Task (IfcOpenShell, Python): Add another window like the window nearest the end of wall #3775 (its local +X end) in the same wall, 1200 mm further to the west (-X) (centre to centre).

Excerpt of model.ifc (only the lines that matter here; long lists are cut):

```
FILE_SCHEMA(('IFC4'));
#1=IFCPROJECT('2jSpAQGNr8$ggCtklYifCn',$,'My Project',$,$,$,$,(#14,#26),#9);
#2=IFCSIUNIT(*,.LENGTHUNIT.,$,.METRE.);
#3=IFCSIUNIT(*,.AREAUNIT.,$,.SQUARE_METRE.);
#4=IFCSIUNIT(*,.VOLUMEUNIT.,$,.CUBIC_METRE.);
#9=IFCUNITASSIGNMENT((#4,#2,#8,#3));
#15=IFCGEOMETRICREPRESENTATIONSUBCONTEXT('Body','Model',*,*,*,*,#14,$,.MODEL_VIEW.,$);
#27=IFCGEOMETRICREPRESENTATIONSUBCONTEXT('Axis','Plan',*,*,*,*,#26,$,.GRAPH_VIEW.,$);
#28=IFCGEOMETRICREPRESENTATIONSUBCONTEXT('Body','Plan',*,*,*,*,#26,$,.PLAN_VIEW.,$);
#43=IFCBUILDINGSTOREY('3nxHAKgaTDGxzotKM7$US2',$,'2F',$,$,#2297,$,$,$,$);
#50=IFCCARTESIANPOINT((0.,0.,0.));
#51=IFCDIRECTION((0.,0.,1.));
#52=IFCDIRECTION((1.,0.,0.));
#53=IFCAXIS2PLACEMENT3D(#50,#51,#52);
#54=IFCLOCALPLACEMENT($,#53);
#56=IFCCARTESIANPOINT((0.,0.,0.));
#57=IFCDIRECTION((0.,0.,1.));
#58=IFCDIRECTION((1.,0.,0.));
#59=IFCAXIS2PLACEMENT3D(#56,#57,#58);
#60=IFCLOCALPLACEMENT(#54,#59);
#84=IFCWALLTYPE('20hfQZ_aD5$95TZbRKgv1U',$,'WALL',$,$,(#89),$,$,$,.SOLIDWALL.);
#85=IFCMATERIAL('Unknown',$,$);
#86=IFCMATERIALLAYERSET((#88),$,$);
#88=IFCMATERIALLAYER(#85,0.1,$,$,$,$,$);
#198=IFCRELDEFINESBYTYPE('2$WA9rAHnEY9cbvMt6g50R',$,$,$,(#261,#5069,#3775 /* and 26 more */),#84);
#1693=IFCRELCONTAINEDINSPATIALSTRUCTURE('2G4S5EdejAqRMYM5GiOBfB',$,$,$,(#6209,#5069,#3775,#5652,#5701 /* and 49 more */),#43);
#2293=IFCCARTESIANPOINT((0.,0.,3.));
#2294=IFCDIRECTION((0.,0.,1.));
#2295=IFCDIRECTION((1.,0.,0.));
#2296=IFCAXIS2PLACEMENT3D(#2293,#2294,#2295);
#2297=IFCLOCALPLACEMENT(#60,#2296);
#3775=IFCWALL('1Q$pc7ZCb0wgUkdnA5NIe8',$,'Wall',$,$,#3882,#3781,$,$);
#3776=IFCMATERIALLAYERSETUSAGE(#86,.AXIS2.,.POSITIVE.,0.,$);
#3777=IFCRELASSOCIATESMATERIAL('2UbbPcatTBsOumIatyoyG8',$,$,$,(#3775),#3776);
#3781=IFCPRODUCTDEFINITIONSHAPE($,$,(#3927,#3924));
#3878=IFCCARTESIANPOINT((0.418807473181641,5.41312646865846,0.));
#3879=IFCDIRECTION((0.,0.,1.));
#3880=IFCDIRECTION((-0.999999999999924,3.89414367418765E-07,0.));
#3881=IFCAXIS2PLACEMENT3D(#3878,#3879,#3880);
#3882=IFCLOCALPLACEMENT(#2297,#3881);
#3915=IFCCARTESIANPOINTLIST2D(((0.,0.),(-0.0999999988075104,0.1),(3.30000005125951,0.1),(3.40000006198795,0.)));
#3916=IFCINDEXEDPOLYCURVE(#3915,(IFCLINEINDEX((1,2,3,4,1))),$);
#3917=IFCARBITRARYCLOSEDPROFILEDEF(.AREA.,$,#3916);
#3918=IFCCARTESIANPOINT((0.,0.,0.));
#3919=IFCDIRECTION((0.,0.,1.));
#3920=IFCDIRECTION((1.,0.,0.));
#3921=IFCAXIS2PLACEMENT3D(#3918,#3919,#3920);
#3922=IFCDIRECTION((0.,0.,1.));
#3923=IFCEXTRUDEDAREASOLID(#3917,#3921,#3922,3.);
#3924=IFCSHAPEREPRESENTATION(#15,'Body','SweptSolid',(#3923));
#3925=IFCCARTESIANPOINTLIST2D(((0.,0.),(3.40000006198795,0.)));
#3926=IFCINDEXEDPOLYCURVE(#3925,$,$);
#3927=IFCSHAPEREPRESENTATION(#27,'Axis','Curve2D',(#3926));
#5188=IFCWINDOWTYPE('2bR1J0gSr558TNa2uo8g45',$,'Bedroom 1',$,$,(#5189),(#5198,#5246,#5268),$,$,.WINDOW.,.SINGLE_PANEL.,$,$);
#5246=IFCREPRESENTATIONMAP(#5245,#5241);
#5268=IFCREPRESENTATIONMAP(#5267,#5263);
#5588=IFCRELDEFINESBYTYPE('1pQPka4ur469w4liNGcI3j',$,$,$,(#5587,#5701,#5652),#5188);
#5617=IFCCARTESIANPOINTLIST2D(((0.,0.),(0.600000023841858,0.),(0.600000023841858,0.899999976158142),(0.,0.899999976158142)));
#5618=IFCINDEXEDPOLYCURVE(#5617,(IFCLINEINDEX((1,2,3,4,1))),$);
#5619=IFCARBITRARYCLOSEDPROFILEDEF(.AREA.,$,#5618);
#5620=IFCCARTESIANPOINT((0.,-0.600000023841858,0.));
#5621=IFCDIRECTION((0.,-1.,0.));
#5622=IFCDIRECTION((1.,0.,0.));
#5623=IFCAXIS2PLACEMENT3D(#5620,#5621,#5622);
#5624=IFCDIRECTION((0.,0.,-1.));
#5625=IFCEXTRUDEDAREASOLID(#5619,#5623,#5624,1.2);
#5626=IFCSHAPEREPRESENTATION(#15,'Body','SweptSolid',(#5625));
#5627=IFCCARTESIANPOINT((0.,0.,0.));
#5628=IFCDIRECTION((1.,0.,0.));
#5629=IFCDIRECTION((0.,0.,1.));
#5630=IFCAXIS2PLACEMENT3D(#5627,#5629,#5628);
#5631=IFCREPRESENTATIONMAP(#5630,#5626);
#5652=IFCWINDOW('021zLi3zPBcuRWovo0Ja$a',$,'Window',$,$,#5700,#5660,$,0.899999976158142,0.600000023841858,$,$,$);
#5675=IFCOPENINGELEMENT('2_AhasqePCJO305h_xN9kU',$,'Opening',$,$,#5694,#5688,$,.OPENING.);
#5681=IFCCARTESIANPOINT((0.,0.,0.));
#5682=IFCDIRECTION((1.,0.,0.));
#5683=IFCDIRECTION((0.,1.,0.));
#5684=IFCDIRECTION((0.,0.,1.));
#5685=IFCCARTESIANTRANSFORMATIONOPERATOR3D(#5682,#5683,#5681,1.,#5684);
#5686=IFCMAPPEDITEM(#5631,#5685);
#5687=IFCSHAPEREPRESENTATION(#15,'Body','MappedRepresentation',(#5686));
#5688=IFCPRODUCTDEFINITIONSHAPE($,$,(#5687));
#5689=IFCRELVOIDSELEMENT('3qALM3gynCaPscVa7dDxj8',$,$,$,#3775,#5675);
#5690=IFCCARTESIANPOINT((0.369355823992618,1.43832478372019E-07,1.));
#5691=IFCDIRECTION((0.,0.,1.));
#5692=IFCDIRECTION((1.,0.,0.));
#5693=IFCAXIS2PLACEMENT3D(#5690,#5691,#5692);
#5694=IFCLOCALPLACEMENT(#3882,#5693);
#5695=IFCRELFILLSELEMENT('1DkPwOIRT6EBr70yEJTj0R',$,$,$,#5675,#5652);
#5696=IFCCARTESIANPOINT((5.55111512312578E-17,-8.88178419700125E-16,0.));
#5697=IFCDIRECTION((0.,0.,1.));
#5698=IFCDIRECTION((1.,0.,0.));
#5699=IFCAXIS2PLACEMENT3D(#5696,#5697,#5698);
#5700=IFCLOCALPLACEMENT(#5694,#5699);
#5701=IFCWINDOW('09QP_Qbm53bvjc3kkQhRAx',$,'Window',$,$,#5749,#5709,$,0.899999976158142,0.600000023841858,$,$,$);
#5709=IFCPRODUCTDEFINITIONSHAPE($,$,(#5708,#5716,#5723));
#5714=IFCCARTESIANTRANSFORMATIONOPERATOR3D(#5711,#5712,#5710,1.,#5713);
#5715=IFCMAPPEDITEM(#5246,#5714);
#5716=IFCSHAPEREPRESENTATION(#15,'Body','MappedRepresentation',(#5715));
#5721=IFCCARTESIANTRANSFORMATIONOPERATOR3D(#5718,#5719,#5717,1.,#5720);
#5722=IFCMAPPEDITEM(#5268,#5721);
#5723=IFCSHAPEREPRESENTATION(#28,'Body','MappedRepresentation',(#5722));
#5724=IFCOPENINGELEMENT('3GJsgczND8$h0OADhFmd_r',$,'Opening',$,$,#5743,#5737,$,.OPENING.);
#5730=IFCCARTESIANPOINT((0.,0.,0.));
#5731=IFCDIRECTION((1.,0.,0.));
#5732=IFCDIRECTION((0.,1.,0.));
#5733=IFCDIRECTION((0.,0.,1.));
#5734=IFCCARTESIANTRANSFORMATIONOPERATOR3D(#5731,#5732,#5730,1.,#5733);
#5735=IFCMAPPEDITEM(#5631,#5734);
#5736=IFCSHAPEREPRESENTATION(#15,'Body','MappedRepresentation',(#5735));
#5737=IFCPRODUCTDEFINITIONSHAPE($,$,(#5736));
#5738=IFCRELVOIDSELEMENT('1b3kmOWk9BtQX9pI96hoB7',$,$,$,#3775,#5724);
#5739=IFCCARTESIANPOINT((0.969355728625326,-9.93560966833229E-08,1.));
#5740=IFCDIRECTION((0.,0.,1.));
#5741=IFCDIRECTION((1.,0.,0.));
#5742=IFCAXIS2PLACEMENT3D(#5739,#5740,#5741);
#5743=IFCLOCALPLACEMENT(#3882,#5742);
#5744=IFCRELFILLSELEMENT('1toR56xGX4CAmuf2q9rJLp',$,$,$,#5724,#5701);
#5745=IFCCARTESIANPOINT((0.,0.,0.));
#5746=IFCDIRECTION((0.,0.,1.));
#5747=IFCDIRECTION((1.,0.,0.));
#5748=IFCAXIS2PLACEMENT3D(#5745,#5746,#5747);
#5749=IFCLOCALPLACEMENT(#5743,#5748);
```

```python
import ifcopenshell
import ifcopenshell.api.feature
import ifcopenshell.api.geometry
import ifcopenshell.api.root
import ifcopenshell.geom
import ifcopenshell.util.element
import ifcopenshell.util.placement
import ifcopenshell.util.shape
import ifcopenshell.util.unit

model = ifcopenshell.open("model.ifc")
unit_scale = ifcopenshell.util.unit.calculate_unit_scale(model)
settings = ifcopenshell.geom.settings()


def volume(element):
    """Net volume in cubic metres, openings subtracted."""
    shape = ifcopenshell.geom.create_shape(settings, element)
    return ifcopenshell.util.shape.get_volume(shape.geometry)


window = model.by_guid("09QP_Qbm53bvjc3kkQhRAx")
opening = window.FillsVoids[0].RelatingOpeningElement
wall = opening.VoidsElements[0].RelatingBuildingElement
before = volume(wall)
shift = ifcopenshell.util.placement.get_local_placement(wall.ObjectPlacement)[:3, 0] * 1.2 / unit_scale

# copy_class copies the void relationship, type, container and properties, but no geometry.
new_opening = ifcopenshell.api.root.copy_class(model, product=opening)
new_opening.Representation = ifcopenshell.util.element.copy_deep(
    model, opening.Representation, exclude=["IfcGeometricRepresentationContext", "IfcRepresentationMap"]
)
new_window = ifcopenshell.api.root.copy_class(model, product=window)
new_window.Representation = ifcopenshell.util.element.copy_deep(
    model, window.Representation, exclude=["IfcGeometricRepresentationContext", "IfcRepresentationMap"]
)
ifcopenshell.api.feature.add_filling(model, opening=new_opening, element=new_window)

for old, new in ((opening, new_opening), (window, new_window)):
    matrix = ifcopenshell.util.placement.get_local_placement(old.ObjectPlacement)
    matrix[:3, 3] += shift
    ifcopenshell.api.geometry.edit_object_placement(model, product=new, matrix=matrix, is_si=False)

after = volume(wall)

print(f"wall volume {before:.3f} -> {after:.3f} m3")

model.write("model_rev.ifc")
```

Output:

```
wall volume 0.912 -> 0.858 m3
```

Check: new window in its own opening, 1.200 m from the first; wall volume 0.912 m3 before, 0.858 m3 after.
